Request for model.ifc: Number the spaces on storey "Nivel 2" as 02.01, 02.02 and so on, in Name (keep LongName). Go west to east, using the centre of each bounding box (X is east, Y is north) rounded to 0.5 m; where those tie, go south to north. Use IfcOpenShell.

First a look at what the model holds.

```python
import ifcopenshell
import ifcopenshell.util.element
import ifcopenshell.util.placement

model = ifcopenshell.open("model.ifc")
print(model.schema)
storey = next(s for s in model.by_type("IfcBuildingStorey") if s.Name == "Nivel 2")
spaces = [e for e in ifcopenshell.util.element.get_decomposition(storey) if e.is_a("IfcSpace")]
for e in sorted(spaces, key=lambda e: e.id()):
    origin = ifcopenshell.util.placement.get_local_placement(e.ObjectPlacement)[:3, 3]
    print(e.id(), e.Name, e.LongName, origin.round(2) + 0.0, sep=" | ")
```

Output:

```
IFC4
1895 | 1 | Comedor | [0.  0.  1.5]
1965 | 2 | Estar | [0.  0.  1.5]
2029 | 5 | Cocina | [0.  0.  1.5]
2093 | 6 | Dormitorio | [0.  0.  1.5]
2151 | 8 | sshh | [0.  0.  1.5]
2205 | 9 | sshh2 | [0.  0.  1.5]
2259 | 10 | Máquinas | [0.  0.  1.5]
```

```python
import ifcopenshell
import ifcopenshell.geom
import ifcopenshell.util.element
import ifcopenshell.util.shape

model = ifcopenshell.open("model.ifc")
settings = ifcopenshell.geom.settings()
settings.set("use-world-coords", True)


def centre(element):
    shape = ifcopenshell.geom.create_shape(settings, element)
    return ifcopenshell.util.shape.get_bbox_centroid(shape.geometry)


storey = next(s for s in model.by_type("IfcBuildingStorey") if s.Name == "Nivel 2")
spaces = [e for e in ifcopenshell.util.element.get_decomposition(storey) if e.is_a("IfcSpace")]

# Insertion points can sit at a corner or the storey origin, so sort by the geometry (in metres).
centres = {e: centre(e) for e in spaces}
spaces.sort(key=lambda e: (round(centres[e][0] / 0.5), centres[e][1]))

for i, e in enumerate(spaces, start=1):
    number = f"02.{i:02d}"
    e.Name = number
    print(e.id(), number)

model.write("model_edited.ifc")
```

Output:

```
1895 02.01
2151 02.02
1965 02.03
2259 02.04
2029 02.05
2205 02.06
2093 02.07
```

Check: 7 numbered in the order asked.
